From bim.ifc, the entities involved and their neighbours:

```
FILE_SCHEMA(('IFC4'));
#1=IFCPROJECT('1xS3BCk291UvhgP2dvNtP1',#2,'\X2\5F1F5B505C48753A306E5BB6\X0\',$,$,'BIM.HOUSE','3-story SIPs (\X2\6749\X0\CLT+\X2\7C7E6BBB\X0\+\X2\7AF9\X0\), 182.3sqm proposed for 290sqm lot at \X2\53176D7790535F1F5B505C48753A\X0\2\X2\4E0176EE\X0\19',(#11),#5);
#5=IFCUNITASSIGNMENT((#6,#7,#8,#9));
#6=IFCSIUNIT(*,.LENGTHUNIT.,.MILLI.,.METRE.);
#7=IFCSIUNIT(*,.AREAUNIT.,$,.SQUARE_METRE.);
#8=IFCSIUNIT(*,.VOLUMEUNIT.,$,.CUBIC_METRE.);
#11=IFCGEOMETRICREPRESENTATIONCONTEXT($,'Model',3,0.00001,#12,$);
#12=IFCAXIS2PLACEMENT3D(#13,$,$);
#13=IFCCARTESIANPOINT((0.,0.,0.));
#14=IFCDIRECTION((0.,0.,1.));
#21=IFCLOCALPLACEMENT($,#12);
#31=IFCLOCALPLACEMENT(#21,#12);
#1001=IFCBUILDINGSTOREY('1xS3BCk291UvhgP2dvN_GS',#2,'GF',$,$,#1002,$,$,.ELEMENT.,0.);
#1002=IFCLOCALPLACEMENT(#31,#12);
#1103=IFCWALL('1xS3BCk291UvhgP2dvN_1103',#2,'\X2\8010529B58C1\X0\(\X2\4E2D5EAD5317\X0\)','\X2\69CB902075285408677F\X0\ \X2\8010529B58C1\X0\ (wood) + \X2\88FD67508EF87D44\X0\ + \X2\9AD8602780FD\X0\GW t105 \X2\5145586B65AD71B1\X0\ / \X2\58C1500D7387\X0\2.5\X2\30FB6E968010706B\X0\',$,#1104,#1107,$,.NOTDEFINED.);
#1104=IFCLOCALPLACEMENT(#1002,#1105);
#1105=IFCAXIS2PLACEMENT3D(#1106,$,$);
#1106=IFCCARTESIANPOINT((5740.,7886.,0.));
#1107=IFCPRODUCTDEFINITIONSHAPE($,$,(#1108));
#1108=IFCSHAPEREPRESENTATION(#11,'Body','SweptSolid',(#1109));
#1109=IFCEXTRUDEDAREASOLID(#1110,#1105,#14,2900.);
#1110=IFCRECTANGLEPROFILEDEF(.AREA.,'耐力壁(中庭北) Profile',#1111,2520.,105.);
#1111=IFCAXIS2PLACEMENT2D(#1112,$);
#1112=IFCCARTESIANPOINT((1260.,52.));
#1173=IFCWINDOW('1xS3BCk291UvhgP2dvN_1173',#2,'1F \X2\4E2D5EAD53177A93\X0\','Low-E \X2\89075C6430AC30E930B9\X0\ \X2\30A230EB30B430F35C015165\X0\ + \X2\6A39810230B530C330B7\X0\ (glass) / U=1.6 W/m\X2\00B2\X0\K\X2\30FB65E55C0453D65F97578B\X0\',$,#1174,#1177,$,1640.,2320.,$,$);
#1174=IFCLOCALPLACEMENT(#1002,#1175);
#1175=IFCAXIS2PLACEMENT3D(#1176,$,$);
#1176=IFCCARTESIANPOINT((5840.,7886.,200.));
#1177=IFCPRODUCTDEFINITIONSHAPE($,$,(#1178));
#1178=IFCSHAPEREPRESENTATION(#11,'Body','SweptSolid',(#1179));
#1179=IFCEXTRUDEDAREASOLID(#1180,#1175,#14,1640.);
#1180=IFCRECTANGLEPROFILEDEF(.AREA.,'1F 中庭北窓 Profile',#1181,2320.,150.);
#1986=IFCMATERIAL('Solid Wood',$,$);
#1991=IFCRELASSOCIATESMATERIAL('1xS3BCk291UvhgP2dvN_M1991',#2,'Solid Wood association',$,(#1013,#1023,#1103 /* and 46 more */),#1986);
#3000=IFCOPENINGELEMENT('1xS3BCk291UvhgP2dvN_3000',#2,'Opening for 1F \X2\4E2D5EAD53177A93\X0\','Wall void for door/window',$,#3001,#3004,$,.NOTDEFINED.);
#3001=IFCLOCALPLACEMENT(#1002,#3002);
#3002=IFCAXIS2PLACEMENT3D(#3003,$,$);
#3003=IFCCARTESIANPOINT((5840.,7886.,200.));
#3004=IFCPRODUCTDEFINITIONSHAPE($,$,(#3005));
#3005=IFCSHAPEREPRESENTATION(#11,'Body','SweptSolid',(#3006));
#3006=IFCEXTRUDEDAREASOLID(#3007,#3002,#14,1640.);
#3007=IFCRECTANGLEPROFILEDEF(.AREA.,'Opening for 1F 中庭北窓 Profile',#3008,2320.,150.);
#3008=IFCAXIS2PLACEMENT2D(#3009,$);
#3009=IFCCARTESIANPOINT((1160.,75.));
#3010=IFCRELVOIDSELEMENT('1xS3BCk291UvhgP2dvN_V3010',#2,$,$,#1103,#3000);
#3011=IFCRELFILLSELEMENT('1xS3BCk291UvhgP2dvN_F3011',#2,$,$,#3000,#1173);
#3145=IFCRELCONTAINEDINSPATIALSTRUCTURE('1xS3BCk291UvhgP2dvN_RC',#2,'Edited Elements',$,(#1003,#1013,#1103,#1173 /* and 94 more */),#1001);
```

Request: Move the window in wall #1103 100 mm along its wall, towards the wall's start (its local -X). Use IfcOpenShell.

```python
import ifcopenshell
import ifcopenshell.api.geometry
import ifcopenshell.util.placement

model = ifcopenshell.open("bim.ifc")

window = model.by_guid("1xS3BCk291UvhgP2dvN_1173")
opening = window.FillsVoids[0].RelatingOpeningElement
wall = opening.VoidsElements[0].RelatingBuildingElement

wall_matrix = ifcopenshell.util.placement.get_local_placement(wall.ObjectPlacement)
shift = wall_matrix[:3, 0] * -100.0
before = ifcopenshell.util.placement.get_local_placement(window.ObjectPlacement)[:3, 3].copy()

# The window is not placed relative to its opening, so move both.
for product in (opening, window):
    matrix = ifcopenshell.util.placement.get_local_placement(product.ObjectPlacement)
    matrix[:3, 3] += shift
    ifcopenshell.api.geometry.edit_object_placement(model, product=product, matrix=matrix, is_si=False)

after = ifcopenshell.util.placement.get_local_placement(window.ObjectPlacement)[:3, 3]
print("window moved by", (after - before).round(3) + 0.0)

model.write("bim_rev.ifc")
```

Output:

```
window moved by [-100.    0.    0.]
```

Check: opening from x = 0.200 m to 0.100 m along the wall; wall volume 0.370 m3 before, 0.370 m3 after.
